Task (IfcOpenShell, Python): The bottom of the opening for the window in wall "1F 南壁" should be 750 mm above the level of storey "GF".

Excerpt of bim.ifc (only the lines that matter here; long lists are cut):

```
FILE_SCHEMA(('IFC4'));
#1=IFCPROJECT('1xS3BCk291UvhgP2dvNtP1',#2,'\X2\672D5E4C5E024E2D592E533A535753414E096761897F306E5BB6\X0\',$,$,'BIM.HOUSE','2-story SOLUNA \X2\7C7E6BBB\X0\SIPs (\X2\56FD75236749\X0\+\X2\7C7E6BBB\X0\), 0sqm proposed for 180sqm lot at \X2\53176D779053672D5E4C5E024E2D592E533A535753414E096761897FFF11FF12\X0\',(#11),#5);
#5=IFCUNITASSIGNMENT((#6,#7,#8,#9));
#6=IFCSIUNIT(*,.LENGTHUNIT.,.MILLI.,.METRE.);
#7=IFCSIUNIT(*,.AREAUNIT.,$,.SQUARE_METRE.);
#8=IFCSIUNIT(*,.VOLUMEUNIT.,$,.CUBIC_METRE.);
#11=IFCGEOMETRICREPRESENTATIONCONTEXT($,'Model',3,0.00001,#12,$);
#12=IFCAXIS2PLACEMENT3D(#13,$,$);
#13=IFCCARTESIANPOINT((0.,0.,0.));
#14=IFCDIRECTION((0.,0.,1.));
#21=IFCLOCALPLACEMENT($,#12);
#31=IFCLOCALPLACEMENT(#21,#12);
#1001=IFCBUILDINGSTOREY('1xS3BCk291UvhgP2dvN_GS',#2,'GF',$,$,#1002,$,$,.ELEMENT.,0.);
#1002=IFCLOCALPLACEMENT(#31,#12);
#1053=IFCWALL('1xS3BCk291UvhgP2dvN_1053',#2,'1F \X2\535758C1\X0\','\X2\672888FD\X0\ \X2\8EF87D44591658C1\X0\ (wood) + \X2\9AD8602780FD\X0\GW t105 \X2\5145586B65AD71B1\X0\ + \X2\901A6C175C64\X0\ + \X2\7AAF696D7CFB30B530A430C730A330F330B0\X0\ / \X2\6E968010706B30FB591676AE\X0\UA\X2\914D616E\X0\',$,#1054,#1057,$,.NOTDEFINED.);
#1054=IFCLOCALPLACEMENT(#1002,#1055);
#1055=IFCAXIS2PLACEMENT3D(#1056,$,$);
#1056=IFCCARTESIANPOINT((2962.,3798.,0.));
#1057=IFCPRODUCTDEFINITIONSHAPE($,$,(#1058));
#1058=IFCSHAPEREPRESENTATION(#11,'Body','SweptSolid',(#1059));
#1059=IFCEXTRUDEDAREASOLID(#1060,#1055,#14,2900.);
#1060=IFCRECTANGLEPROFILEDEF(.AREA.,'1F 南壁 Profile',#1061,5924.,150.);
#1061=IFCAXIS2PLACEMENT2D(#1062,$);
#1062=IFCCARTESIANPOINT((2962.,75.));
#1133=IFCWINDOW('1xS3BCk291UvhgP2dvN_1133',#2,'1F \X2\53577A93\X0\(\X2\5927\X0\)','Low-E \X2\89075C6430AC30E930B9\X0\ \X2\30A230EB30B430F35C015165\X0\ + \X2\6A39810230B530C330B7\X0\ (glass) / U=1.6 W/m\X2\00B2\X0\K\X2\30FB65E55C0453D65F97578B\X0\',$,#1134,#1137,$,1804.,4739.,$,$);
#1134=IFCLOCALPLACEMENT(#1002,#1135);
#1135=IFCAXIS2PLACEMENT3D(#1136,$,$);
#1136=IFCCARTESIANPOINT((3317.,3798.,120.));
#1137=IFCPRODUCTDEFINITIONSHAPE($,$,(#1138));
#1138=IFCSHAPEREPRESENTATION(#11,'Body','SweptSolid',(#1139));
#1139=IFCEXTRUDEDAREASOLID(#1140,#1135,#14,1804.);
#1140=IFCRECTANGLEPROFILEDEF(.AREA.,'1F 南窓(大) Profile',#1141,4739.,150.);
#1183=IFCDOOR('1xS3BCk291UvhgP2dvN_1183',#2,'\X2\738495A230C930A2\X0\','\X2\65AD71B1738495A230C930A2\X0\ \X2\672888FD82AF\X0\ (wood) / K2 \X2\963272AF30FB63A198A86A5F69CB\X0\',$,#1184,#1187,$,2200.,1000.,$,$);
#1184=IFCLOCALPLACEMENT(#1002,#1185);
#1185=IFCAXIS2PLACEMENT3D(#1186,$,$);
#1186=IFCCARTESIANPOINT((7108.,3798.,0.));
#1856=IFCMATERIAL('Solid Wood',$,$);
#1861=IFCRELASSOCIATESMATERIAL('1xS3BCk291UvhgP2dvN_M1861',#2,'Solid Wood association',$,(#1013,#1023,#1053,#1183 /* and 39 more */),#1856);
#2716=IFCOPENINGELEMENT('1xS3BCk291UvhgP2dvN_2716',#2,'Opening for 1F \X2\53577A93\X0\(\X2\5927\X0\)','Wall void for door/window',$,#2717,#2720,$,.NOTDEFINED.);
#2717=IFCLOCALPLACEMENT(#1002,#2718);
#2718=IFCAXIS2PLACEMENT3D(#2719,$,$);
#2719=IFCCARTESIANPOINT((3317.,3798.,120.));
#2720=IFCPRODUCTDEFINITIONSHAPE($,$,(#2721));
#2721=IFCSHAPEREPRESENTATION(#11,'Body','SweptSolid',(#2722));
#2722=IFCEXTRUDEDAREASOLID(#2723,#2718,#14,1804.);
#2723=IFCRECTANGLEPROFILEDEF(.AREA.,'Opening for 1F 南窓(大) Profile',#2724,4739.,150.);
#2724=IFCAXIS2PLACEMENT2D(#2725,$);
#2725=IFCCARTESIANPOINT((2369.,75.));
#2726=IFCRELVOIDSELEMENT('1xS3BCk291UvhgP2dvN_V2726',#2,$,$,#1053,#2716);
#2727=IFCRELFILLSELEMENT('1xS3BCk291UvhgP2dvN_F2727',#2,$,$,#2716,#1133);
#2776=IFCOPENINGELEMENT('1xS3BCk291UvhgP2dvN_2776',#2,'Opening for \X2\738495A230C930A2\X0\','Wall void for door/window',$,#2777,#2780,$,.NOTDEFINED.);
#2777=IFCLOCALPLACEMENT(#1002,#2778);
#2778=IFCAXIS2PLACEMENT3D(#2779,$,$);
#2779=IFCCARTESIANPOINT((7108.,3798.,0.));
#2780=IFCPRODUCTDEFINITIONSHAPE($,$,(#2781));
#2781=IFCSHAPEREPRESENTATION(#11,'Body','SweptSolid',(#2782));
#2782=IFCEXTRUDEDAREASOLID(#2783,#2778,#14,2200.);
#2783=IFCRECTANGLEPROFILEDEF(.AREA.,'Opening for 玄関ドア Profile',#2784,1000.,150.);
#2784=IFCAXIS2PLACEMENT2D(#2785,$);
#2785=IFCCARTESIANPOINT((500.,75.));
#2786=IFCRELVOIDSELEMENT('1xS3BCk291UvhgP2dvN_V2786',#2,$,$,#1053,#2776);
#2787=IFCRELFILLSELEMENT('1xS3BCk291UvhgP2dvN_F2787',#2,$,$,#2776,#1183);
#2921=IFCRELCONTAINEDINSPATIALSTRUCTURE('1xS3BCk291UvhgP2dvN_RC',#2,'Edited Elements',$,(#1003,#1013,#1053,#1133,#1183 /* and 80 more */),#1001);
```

```python
import numpy as np
import ifcopenshell
import ifcopenshell.api.geometry
import ifcopenshell.geom
import ifcopenshell.util.element
import ifcopenshell.util.placement
import ifcopenshell.util.shape
import ifcopenshell.util.unit

model = ifcopenshell.open("bim.ifc")
unit_scale = ifcopenshell.util.unit.calculate_unit_scale(model)

window = model.by_guid("1xS3BCk291UvhgP2dvN_1133")
opening = window.FillsVoids[0].RelatingOpeningElement
storey = ifcopenshell.util.element.get_container(window, ifc_class="IfcBuildingStorey")
level = ifcopenshell.util.placement.get_local_placement(storey.ObjectPlacement)[2, 3]

# The opening's origin need not be at the sill, so measure its lowest point.
shape = ifcopenshell.geom.create_shape(ifcopenshell.geom.settings(), opening)
bottom = ifcopenshell.util.shape.get_shape_bottom_elevation(shape, shape.geometry) / unit_scale
dz = level + 750.0 - bottom

shift = np.array([0.0, 0.0, dz])
# The window is not placed relative to its opening, so move both.
for product in (opening, window):
    matrix = ifcopenshell.util.placement.get_local_placement(product.ObjectPlacement)
    matrix[:3, 3] += shift
    ifcopenshell.api.geometry.edit_object_placement(model, product=product, matrix=matrix, is_si=False)

print(f"moved by {dz * unit_scale:+.3f} m")

model.write("bim_updated.ifc")
```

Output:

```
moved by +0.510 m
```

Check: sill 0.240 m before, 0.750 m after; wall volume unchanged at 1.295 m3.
